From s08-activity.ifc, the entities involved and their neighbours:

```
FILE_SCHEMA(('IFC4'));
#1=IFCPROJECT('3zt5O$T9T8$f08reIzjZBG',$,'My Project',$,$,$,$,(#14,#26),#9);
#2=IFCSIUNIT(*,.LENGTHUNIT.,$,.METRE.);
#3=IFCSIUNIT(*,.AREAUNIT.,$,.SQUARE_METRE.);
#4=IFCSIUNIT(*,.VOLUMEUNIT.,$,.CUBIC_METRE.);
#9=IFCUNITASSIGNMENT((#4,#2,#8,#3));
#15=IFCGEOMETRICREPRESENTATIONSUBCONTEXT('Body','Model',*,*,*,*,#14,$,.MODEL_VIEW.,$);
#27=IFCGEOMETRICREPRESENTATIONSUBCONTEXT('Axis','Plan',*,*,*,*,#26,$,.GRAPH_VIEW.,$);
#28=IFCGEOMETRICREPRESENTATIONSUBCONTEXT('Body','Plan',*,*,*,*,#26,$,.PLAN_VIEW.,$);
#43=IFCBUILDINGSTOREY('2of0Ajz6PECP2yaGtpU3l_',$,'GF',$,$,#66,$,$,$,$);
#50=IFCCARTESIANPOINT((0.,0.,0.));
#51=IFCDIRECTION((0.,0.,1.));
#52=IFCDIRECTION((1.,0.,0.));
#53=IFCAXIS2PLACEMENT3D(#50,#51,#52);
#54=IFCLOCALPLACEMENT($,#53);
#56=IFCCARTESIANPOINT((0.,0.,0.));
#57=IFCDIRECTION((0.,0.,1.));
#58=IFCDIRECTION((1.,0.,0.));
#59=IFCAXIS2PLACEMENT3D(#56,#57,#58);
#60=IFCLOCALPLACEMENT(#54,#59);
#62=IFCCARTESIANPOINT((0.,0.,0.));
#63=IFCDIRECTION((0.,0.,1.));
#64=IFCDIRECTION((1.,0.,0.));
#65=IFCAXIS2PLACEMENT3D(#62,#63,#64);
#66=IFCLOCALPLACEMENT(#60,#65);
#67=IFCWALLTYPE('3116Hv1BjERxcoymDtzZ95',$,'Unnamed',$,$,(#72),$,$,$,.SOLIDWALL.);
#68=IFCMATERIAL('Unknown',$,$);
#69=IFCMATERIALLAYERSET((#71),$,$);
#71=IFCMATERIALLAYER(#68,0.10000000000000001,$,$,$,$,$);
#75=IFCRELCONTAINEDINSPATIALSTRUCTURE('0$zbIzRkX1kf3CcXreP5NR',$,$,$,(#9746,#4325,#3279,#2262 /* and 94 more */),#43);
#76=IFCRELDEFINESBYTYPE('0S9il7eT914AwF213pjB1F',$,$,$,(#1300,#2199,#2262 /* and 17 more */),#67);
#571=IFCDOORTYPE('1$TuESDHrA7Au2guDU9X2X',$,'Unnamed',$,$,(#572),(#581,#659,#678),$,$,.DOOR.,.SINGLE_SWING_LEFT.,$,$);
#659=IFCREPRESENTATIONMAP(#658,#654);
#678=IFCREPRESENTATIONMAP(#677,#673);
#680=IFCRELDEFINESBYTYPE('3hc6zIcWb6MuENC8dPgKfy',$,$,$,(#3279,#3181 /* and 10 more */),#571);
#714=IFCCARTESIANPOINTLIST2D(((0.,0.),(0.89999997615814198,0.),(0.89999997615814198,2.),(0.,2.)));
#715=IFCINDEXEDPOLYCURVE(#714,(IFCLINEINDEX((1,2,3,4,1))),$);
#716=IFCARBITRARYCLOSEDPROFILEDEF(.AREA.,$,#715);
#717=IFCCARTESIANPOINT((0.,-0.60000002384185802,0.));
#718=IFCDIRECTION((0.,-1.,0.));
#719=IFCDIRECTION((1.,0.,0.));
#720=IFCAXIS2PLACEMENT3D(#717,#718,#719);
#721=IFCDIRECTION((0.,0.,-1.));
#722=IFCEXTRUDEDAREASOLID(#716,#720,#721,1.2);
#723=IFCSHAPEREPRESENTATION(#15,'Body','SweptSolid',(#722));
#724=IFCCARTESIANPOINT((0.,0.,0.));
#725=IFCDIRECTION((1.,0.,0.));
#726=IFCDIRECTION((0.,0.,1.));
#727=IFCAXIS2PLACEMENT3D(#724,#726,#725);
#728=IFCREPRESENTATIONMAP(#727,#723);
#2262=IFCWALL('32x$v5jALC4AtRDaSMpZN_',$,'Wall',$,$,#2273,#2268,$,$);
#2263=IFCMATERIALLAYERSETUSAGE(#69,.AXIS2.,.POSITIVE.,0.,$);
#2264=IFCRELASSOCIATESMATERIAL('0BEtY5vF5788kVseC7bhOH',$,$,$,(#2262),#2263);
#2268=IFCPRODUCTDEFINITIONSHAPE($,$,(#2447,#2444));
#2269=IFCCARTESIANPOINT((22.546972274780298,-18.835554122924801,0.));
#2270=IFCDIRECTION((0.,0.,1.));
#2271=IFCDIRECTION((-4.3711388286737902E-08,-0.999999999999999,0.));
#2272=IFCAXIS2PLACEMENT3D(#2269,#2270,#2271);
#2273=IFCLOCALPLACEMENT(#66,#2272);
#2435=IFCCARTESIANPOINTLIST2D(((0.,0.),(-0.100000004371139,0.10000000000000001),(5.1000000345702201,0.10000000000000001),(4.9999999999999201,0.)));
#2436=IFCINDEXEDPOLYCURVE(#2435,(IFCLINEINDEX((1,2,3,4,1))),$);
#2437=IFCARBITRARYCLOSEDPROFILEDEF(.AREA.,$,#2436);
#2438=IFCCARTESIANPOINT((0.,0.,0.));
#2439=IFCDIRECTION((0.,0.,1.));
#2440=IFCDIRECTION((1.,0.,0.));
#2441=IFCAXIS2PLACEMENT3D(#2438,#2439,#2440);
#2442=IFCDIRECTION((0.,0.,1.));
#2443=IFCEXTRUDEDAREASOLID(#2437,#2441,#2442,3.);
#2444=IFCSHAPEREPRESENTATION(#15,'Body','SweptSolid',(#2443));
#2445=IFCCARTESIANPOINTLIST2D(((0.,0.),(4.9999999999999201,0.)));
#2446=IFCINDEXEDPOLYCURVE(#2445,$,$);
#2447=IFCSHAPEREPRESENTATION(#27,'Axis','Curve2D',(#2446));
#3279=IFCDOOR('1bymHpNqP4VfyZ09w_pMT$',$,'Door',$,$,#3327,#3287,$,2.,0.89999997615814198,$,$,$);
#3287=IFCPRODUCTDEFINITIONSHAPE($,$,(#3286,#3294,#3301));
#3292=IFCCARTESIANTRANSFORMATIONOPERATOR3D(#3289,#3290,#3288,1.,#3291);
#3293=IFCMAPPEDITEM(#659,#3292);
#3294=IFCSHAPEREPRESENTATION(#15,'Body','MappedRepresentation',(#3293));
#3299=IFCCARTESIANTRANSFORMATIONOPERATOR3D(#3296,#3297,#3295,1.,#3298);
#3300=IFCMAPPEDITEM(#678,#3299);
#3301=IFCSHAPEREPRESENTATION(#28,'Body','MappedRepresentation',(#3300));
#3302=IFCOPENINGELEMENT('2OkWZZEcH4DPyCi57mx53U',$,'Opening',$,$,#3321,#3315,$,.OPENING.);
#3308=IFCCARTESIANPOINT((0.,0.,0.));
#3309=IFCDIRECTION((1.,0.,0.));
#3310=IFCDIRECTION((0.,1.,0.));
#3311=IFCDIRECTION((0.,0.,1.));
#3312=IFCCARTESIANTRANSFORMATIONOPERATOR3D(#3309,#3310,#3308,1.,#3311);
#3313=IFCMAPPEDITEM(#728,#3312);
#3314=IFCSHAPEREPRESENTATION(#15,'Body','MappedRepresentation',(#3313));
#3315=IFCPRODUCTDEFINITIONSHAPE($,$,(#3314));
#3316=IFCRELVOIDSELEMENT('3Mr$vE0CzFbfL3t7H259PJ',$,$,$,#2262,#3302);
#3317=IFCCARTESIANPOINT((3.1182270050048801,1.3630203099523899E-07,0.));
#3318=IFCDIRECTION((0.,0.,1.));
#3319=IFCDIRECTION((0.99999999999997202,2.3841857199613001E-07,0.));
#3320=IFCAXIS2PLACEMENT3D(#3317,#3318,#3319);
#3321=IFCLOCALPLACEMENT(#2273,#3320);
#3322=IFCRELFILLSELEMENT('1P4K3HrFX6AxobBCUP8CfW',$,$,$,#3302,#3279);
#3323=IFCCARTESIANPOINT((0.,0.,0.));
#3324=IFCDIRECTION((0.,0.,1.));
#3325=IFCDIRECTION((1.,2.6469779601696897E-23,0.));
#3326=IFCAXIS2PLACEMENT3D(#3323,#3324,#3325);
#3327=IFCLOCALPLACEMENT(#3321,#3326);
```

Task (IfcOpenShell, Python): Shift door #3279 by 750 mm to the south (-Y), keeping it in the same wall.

```python
import ifcopenshell
import ifcopenshell.api.geometry
import ifcopenshell.util.placement
import ifcopenshell.util.unit

model = ifcopenshell.open("s08-activity.ifc")
unit_scale = ifcopenshell.util.unit.calculate_unit_scale(model)

door = model.by_guid("1bymHpNqP4VfyZ09w_pMT$")
opening = door.FillsVoids[0].RelatingOpeningElement
wall = opening.VoidsElements[0].RelatingBuildingElement

wall_matrix = ifcopenshell.util.placement.get_local_placement(wall.ObjectPlacement)
shift = wall_matrix[:3, 0] * 0.75 / unit_scale
before = ifcopenshell.util.placement.get_local_placement(door.ObjectPlacement)[:3, 3].copy()

# The door is placed relative to its opening, so it follows when the opening moves.
matrix = ifcopenshell.util.placement.get_local_placement(opening.ObjectPlacement)
matrix[:3, 3] += shift
ifcopenshell.api.geometry.edit_object_placement(
    model, product=opening, matrix=matrix, is_si=False, should_transform_children=True
)

after = ifcopenshell.util.placement.get_local_placement(door.ObjectPlacement)[:3, 3]
print("door moved by", (after - before).round(3) + 0.0)

model.write("s08-activity_updated.ifc")
```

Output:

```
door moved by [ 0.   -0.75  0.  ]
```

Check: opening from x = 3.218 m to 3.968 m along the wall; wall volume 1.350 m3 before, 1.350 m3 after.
